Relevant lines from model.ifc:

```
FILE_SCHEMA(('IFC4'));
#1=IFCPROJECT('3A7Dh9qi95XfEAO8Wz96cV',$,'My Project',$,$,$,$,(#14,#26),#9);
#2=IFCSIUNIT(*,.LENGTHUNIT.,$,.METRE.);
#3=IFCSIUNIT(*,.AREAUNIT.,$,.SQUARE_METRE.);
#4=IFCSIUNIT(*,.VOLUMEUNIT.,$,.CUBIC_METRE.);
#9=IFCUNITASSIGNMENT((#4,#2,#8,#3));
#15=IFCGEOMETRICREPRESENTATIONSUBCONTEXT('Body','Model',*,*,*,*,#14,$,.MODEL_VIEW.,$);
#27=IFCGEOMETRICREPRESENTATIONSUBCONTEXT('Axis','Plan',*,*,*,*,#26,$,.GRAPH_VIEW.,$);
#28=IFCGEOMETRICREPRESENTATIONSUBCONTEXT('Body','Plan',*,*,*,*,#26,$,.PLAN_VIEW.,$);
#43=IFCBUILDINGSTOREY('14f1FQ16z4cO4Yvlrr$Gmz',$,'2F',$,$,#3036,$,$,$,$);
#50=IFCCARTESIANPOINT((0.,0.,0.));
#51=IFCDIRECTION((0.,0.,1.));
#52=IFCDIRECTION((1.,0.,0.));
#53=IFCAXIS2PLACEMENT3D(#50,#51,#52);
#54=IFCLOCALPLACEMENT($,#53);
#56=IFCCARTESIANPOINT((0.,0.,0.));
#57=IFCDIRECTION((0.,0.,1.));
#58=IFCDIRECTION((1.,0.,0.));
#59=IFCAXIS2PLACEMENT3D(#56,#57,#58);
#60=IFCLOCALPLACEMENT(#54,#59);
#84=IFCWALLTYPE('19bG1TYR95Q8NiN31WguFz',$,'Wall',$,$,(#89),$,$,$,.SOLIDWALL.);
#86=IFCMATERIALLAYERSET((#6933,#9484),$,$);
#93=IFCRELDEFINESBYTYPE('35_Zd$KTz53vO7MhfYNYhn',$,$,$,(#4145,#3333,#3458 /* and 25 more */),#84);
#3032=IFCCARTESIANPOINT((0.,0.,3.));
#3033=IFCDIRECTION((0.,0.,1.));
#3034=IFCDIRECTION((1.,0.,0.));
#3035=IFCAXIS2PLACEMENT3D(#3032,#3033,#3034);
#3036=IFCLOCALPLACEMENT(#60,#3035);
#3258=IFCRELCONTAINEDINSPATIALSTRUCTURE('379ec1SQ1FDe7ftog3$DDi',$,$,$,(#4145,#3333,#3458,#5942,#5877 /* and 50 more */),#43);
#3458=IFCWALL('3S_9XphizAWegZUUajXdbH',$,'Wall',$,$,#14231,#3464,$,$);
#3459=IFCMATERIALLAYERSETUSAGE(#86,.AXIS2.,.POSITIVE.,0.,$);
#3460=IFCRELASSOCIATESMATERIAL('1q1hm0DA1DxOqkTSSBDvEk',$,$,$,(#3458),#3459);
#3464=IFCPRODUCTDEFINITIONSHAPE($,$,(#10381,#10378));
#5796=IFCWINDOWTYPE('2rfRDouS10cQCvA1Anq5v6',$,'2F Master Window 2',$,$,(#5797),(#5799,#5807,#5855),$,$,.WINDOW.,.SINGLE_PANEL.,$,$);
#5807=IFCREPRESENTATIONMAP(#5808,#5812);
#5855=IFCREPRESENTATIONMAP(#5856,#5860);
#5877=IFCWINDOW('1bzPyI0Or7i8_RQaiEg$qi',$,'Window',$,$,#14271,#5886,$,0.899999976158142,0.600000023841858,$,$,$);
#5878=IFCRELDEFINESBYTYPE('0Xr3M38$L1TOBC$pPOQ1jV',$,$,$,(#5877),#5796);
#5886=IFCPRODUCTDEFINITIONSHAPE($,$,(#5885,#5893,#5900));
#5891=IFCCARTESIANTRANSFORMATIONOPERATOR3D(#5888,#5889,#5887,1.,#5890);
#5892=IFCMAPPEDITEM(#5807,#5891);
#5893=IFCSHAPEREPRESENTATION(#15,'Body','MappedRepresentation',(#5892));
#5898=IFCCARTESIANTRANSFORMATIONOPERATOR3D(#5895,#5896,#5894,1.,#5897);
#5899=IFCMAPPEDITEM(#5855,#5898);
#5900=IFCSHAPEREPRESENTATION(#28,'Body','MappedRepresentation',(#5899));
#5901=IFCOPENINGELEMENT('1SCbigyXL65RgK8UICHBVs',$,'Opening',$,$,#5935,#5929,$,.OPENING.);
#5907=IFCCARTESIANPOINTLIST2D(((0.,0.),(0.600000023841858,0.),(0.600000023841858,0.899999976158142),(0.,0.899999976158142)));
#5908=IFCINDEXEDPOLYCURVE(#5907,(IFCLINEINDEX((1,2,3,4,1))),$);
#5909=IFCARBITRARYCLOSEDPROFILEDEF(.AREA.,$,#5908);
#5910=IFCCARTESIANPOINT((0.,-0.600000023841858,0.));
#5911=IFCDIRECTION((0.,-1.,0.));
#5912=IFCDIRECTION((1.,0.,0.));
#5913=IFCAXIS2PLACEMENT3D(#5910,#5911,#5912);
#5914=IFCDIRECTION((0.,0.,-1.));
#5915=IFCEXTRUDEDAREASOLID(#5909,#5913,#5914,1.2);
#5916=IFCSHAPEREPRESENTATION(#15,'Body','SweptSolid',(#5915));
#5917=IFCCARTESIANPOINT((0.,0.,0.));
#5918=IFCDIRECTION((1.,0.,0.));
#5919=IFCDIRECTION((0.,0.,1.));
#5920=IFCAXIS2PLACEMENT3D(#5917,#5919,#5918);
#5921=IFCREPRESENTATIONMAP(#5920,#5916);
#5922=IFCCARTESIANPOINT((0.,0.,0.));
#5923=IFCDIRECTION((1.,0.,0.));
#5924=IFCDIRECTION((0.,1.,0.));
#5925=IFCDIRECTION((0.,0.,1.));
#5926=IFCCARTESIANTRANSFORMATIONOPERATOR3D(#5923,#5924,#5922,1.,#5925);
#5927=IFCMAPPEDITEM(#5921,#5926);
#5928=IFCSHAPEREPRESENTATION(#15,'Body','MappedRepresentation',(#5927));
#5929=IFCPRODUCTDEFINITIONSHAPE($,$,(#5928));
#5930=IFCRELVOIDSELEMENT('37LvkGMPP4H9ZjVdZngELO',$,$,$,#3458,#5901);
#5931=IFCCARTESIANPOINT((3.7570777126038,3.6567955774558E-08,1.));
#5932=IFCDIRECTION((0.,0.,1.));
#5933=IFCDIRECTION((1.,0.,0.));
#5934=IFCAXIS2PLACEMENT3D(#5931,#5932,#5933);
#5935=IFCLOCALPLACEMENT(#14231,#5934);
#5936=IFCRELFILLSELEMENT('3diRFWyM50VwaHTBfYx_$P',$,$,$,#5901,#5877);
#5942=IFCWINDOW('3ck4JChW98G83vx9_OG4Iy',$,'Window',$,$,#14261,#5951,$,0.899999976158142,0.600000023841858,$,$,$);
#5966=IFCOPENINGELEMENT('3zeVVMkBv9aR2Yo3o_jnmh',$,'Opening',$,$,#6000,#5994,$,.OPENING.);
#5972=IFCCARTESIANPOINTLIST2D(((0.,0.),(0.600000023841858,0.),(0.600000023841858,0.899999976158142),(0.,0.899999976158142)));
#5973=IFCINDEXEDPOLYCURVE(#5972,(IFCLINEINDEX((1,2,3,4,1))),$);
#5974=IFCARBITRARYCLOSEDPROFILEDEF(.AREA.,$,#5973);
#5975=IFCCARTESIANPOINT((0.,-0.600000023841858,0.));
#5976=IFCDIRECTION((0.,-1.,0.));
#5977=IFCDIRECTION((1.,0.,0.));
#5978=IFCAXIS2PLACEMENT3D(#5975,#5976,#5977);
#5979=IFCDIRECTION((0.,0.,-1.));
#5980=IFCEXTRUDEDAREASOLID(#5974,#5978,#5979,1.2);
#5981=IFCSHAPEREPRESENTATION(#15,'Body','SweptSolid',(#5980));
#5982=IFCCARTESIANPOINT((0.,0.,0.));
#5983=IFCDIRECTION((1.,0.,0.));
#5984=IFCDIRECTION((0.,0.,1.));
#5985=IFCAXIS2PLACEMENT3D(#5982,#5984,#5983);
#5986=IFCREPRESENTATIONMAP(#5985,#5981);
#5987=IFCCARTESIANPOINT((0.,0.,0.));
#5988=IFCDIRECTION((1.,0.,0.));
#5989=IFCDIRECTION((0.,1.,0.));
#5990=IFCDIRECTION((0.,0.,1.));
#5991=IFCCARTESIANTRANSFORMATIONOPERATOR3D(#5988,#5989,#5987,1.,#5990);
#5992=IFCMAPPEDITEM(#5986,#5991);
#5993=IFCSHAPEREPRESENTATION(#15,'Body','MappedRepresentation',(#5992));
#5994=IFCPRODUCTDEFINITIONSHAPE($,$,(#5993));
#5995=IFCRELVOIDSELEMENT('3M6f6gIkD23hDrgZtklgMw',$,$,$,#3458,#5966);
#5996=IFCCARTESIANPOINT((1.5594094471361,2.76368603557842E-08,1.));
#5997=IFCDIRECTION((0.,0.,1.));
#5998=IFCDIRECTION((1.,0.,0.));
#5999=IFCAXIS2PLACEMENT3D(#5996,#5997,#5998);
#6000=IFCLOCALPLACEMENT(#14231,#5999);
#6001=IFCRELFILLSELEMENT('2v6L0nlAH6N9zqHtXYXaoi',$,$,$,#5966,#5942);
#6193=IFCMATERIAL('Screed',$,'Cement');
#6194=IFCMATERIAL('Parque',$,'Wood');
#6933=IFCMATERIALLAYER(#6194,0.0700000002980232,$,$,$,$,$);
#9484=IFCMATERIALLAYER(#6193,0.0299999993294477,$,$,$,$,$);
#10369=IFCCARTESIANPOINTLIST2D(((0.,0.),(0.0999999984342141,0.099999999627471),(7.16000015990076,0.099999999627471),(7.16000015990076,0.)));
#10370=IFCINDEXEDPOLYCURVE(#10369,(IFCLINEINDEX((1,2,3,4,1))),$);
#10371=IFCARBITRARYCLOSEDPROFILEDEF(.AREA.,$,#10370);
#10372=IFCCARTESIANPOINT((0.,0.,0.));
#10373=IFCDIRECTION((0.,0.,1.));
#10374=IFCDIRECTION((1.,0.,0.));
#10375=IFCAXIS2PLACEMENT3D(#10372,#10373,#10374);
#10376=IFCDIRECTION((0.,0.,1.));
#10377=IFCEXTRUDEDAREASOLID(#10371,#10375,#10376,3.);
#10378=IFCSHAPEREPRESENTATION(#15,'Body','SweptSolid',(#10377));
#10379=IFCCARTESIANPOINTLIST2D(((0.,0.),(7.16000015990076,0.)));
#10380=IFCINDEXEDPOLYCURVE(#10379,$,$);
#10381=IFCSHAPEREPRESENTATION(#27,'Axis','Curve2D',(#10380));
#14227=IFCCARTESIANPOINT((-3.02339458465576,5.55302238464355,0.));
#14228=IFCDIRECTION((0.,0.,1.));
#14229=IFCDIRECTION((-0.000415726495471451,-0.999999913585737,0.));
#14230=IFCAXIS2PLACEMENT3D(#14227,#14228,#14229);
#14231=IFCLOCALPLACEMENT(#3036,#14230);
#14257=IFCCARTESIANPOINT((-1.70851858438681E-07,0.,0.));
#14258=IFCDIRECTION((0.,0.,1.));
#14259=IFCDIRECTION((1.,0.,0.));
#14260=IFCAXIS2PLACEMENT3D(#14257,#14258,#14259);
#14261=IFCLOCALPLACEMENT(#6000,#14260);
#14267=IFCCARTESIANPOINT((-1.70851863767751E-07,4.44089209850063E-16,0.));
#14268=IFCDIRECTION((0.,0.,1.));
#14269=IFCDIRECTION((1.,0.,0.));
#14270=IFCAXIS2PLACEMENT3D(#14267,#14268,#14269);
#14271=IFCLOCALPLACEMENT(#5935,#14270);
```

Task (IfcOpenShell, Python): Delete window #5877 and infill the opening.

```python
import ifcopenshell
import ifcopenshell.api.feature
import ifcopenshell.api.root
import ifcopenshell.geom
import ifcopenshell.util.shape

model = ifcopenshell.open("model.ifc")
settings = ifcopenshell.geom.settings()


def volume(element):
    """Net volume in cubic metres, openings subtracted."""
    shape = ifcopenshell.geom.create_shape(settings, element)
    return ifcopenshell.util.shape.get_volume(shape.geometry)


window = model.by_id(5877)
opening = window.FillsVoids[0].RelatingOpeningElement
wall = opening.VoidsElements[0].RelatingBuildingElement
before = volume(wall)

ifcopenshell.api.root.remove_product(model, product=window)
ifcopenshell.api.feature.remove_feature(model, feature=opening)

after = volume(wall)

print(f"wall volume {before:.3f} -> {after:.3f} m3")

model.write("model_rev.ifc")
```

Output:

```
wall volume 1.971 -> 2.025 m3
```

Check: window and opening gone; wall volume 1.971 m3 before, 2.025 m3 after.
